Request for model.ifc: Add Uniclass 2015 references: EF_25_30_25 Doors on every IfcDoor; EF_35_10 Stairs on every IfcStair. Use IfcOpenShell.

First a look at what the model holds.

```python
import ifcopenshell

model = ifcopenshell.open("model.ifc")
print(model.schema)
print("classifications:", [c.Name for c in model.by_type("IfcClassification")])
for ifc_class in ("IfcDoor", "IfcRoof", "IfcStair", "IfcWall", "IfcWindow"):
    print(ifc_class, len(model.by_type(ifc_class)))
```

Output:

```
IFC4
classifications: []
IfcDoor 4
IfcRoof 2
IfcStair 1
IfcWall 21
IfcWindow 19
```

```python
import ifcopenshell
import ifcopenshell.api.classification

model = ifcopenshell.open("model.ifc")

system = ifcopenshell.api.classification.add_classification(model, classification="Uniclass 2015")

codes = {
    "IfcDoor": ("EF_25_30_25", "Doors"),
    "IfcStair": ("EF_35_10", "Stairs"),
}
for ifc_class, (code, name) in codes.items():
    products = model.by_type(ifc_class)
    ifcopenshell.api.classification.add_reference(
        model, products=products, classification=system, identification=code, name=name
    )
    print(code, len(products))

model.write("model_rev.ifc")
```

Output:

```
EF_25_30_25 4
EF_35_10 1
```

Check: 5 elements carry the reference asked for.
